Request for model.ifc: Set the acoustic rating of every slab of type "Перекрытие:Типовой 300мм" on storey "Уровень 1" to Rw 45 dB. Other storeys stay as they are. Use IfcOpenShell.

First a look at what the model holds.

```python
import ifcopenshell
import ifcopenshell.util.element

model = ifcopenshell.open("model.ifc")
print(model.schema)
storey = next(s for s in model.by_type("IfcBuildingStorey") if s.Name == "Уровень 1")
slabs = [e for e in ifcopenshell.util.element.get_decomposition(storey) if e.is_a("IfcSlab")]
seen = {}
for e in slabs:
    element_type = ifcopenshell.util.element.get_type(e)
    key = (element_type.Name if element_type != e and element_type else None, ifcopenshell.util.element.get_pset(e, "Pset_SlabCommon", "AcousticRating"))
    seen[key] = seen.get(key, 0) + 1
for (name, value), count in sorted(seen.items(), key=str):
    print(count, "x", name, "|", value)
```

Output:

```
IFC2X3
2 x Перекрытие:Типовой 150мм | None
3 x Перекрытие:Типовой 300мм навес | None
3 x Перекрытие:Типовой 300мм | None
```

```python
import ifcopenshell
import ifcopenshell.api.pset
import ifcopenshell.util.element

model = ifcopenshell.open("model.ifc")

storey = next(s for s in model.by_type("IfcBuildingStorey") if s.Name == "Уровень 1")
slabs = [e for e in ifcopenshell.util.element.get_decomposition(storey) if e.is_a("IfcSlab")]

count = 0
for e in slabs:
    element_type = ifcopenshell.util.element.get_type(e)
    if element_type in (None, e) or element_type.Name != "Перекрытие:Типовой 300мм":
        continue
    # add_pset returns the element's existing set when there is one.
    pset = ifcopenshell.api.pset.add_pset(model, product=e, name="Pset_SlabCommon")
    ifcopenshell.api.pset.edit_pset(model, pset=pset, properties={"AcousticRating": "Rw 45 dB"})
    count += 1

print(count, "slabs updated")

model.write("model_edited.ifc")
```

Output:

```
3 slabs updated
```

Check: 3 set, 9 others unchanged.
